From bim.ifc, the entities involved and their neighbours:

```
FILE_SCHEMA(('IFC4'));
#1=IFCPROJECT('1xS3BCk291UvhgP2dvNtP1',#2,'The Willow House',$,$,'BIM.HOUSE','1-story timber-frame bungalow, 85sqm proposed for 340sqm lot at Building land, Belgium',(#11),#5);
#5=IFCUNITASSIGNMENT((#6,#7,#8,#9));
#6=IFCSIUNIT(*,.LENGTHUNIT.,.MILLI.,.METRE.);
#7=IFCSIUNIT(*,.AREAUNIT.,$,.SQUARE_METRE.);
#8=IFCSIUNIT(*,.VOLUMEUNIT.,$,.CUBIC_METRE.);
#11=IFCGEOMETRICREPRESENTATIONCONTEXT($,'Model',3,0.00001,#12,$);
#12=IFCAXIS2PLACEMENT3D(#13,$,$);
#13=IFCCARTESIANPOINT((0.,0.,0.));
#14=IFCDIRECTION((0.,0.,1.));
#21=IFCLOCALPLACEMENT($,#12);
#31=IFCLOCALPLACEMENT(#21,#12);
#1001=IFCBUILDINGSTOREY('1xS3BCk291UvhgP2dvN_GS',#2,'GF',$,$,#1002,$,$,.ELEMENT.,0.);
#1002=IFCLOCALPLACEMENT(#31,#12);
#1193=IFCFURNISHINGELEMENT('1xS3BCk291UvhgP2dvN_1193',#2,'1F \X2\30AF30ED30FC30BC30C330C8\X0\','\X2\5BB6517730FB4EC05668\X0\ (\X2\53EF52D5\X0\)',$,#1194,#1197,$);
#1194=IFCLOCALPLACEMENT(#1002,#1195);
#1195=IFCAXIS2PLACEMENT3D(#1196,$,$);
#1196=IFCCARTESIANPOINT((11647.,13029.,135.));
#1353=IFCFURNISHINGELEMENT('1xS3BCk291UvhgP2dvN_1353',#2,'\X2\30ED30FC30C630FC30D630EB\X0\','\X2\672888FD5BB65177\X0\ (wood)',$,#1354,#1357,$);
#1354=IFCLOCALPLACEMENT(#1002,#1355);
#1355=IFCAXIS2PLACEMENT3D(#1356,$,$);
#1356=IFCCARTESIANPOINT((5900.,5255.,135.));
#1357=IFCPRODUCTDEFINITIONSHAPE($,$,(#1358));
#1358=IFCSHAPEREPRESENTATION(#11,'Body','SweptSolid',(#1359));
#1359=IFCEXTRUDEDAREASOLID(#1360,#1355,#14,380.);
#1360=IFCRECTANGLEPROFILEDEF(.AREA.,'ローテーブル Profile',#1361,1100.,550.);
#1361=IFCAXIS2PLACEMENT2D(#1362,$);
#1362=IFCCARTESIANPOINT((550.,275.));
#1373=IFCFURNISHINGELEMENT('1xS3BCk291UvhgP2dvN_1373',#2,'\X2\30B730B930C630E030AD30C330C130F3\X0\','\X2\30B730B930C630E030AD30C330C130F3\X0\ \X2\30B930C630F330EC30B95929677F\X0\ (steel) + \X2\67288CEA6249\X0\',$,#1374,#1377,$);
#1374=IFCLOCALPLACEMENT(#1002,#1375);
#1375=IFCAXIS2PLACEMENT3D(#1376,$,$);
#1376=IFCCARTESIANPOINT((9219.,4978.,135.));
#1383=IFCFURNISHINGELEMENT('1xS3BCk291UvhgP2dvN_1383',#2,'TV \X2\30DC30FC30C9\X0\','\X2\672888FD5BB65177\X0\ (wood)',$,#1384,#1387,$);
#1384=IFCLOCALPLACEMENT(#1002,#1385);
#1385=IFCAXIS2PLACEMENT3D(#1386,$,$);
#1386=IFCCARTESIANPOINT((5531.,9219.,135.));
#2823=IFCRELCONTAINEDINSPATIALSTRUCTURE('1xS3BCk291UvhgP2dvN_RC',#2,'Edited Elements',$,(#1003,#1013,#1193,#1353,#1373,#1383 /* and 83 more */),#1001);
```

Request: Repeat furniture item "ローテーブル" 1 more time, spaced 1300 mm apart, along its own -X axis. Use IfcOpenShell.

```python
import ifcopenshell
import ifcopenshell.api.geometry
import ifcopenshell.api.root
import ifcopenshell.util.element
import ifcopenshell.util.placement

model = ifcopenshell.open("bim.ifc")


def reuse_history(source, copy):
    """copy_class also copies each property set's owner history, people and application; keep the originals."""
    for rel in copy.IsDefinedBy:
        if rel.is_a("IfcRelDefinesByProperties") and (history := rel.RelatingPropertyDefinition.OwnerHistory):
            rel.RelatingPropertyDefinition.OwnerHistory = source.OwnerHistory
            ifcopenshell.util.element.remove_deep2(model, history)


source = model.by_guid("1xS3BCk291UvhgP2dvN_1353")
base = ifcopenshell.util.placement.get_local_placement(source.ObjectPlacement)
step = -base[:3, 0] * 1300.0

for i in range(1, 2):
    copy = ifcopenshell.api.root.copy_class(model, product=source)
    copy.Representation = ifcopenshell.util.element.copy_deep(
        model, source.Representation, exclude=["IfcGeometricRepresentationContext", "IfcRepresentationMap"]
    )
    reuse_history(source, copy)
    matrix = base.copy()
    matrix[:3, 3] += i * step
    print("added at", matrix[:3, 3].round(3) + 0.0)
    ifcopenshell.api.geometry.edit_object_placement(model, product=copy, matrix=matrix, is_si=False)

model.write("bim_edited.ifc")
```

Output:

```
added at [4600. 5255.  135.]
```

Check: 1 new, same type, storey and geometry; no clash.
